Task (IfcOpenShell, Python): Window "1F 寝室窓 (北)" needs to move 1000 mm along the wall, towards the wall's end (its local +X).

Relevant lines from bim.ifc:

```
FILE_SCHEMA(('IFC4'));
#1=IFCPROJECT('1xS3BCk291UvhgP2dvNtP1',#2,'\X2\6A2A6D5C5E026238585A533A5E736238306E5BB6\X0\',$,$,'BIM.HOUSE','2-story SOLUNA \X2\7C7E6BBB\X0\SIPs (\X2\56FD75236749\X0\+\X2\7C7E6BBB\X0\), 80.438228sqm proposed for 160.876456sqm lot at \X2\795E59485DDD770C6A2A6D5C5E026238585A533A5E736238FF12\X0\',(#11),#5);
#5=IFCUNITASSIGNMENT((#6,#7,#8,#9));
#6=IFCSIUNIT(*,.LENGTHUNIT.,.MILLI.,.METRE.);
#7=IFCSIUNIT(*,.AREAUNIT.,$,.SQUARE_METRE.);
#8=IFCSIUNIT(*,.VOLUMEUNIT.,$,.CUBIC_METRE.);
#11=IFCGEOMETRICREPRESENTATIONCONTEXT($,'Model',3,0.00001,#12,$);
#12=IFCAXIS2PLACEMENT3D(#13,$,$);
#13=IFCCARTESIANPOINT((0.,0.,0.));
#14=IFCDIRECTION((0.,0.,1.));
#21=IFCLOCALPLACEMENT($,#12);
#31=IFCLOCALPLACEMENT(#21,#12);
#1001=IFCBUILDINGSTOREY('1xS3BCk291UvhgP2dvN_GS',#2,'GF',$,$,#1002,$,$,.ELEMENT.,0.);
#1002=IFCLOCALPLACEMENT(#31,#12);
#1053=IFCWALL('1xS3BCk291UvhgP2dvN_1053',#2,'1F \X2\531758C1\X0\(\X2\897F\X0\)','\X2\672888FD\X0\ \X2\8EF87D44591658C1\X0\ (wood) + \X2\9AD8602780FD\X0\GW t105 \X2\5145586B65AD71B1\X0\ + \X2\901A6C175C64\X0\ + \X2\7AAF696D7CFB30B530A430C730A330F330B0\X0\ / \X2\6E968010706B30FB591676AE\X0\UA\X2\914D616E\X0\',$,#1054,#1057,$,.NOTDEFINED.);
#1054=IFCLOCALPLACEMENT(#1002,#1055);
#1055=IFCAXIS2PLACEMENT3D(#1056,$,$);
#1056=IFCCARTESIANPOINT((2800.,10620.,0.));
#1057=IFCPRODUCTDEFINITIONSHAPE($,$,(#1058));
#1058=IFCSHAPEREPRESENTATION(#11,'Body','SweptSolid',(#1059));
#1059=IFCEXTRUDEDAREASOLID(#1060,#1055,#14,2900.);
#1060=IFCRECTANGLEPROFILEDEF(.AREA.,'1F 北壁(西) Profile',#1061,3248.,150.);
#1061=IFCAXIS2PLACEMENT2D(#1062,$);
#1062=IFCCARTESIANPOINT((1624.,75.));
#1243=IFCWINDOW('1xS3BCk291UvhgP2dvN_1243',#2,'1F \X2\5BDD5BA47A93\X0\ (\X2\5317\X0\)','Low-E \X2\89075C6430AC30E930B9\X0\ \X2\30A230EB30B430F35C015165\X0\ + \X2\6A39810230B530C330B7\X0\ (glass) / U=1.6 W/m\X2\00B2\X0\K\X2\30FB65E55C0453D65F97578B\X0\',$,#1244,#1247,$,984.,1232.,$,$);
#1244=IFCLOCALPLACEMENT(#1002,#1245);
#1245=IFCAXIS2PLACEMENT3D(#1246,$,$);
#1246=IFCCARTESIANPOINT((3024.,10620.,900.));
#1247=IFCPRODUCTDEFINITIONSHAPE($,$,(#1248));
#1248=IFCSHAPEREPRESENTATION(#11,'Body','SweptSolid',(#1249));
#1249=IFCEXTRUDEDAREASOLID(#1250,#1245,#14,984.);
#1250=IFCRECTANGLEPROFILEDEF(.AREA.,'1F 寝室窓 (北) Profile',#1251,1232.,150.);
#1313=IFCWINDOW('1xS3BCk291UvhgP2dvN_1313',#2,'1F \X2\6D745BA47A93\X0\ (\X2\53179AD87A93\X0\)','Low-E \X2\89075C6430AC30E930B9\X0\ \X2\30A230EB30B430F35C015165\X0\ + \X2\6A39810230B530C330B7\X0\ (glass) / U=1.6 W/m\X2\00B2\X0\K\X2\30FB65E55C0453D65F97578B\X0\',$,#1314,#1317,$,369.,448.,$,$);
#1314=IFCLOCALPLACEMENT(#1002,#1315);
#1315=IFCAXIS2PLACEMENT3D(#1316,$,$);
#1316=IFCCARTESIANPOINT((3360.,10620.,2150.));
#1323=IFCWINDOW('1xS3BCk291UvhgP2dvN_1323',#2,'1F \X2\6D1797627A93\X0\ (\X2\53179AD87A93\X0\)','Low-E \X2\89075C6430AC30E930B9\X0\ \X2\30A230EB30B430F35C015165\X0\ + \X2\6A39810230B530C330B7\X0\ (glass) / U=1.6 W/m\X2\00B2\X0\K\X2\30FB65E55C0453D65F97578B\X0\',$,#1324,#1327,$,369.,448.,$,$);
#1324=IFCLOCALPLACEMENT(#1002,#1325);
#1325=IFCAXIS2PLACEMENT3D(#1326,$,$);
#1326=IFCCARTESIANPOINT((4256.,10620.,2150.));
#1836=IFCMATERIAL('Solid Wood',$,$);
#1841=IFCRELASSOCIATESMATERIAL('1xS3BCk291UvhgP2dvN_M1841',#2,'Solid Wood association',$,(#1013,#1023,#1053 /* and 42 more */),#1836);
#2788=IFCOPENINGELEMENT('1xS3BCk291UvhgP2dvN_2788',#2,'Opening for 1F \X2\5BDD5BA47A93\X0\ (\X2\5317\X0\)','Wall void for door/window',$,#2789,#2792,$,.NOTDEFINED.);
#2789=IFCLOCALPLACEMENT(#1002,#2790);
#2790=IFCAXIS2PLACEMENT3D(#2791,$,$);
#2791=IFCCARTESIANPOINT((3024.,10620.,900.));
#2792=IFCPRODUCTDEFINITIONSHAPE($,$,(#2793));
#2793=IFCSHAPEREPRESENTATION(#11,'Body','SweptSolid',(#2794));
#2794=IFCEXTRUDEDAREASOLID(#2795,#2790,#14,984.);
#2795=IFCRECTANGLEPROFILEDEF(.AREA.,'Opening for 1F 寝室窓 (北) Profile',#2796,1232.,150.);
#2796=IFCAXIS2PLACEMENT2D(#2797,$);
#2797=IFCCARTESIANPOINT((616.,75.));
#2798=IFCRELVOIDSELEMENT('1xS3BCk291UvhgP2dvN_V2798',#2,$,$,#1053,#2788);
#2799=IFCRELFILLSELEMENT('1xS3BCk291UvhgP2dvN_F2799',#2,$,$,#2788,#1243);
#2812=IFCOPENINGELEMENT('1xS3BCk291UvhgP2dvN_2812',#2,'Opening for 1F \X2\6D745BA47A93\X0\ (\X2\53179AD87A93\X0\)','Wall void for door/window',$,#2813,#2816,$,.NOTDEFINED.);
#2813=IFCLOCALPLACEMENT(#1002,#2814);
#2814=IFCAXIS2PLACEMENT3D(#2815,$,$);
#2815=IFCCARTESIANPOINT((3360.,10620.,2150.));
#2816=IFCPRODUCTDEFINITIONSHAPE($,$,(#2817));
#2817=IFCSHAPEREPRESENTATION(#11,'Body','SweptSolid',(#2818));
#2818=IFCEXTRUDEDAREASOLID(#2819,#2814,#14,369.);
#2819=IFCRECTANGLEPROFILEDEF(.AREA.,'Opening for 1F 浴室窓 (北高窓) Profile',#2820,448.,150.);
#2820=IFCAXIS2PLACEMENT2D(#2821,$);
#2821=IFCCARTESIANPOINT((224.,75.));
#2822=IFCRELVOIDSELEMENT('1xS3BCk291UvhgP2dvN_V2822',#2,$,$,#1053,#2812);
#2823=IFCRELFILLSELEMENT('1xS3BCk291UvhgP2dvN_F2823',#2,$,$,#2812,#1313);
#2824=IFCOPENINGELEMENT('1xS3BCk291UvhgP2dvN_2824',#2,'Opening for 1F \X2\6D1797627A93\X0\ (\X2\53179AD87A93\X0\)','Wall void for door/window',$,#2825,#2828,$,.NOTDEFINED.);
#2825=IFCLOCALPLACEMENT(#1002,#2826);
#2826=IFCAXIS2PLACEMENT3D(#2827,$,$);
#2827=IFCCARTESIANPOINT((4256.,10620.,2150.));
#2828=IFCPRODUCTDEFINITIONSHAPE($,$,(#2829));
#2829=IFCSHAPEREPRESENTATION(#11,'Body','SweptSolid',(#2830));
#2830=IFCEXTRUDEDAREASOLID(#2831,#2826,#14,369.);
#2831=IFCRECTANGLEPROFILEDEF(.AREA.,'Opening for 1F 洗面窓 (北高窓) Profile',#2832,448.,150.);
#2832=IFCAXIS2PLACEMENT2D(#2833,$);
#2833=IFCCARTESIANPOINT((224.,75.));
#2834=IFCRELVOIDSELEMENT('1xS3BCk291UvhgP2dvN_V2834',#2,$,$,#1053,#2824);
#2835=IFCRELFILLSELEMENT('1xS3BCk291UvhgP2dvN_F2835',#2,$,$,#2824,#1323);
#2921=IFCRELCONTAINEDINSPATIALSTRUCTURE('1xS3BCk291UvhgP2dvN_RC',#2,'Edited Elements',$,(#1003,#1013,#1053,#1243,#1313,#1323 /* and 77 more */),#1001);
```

```python
import ifcopenshell
import ifcopenshell.api.geometry
import ifcopenshell.util.placement
import ifcopenshell.util.unit

model = ifcopenshell.open("bim.ifc")
unit_scale = ifcopenshell.util.unit.calculate_unit_scale(model)

window = model.by_guid("1xS3BCk291UvhgP2dvN_1243")
opening = window.FillsVoids[0].RelatingOpeningElement
wall = opening.VoidsElements[0].RelatingBuildingElement

wall_matrix = ifcopenshell.util.placement.get_local_placement(wall.ObjectPlacement)
shift = wall_matrix[:3, 0] * 1 / unit_scale
before = ifcopenshell.util.placement.get_local_placement(window.ObjectPlacement)[:3, 3].copy()

# The window is not placed relative to its opening, so move both.
for product in (opening, window):
    matrix = ifcopenshell.util.placement.get_local_placement(product.ObjectPlacement)
    matrix[:3, 3] += shift
    ifcopenshell.api.geometry.edit_object_placement(model, product=product, matrix=matrix, is_si=False)

after = ifcopenshell.util.placement.get_local_placement(window.ObjectPlacement)[:3, 3]
print("window moved by", (after - before).round(3) + 0.0)

model.write("bim_edited.ifc")
```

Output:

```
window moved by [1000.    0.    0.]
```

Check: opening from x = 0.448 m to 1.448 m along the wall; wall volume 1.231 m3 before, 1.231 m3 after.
